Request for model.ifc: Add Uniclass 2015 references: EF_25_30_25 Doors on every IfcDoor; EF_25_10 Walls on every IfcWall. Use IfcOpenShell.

First a look at what the model holds.

```python
import ifcopenshell

model = ifcopenshell.open("model.ifc")
print(model.schema)
print("classifications:", [c.Name for c in model.by_type("IfcClassification")])
for ifc_class in ("IfcDoor", "IfcRoof", "IfcStair", "IfcWall", "IfcWindow"):
    print(ifc_class, len(model.by_type(ifc_class)))
```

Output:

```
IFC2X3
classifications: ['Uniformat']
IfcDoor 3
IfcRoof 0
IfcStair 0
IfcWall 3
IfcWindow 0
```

```python
import ifcopenshell
import ifcopenshell.api.classification

model = ifcopenshell.open("model.ifc")

# IFC2X3 requires Source and Edition and has no link from the project to the system.
system = model.create_entity("IfcClassification", Source="NBS", Edition="2015", Name="Uniclass 2015")

codes = {
    "IfcDoor": ("EF_25_30_25", "Doors"),
    "IfcWall": ("EF_25_10", "Walls"),
}
for ifc_class, (code, name) in codes.items():
    products = model.by_type(ifc_class)
    ifcopenshell.api.classification.add_reference(
        model, products=products, classification=system, identification=code, name=name
    )
    print(code, len(products))

model.write("model-out.ifc")
```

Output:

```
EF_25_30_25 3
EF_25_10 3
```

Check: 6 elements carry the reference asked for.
